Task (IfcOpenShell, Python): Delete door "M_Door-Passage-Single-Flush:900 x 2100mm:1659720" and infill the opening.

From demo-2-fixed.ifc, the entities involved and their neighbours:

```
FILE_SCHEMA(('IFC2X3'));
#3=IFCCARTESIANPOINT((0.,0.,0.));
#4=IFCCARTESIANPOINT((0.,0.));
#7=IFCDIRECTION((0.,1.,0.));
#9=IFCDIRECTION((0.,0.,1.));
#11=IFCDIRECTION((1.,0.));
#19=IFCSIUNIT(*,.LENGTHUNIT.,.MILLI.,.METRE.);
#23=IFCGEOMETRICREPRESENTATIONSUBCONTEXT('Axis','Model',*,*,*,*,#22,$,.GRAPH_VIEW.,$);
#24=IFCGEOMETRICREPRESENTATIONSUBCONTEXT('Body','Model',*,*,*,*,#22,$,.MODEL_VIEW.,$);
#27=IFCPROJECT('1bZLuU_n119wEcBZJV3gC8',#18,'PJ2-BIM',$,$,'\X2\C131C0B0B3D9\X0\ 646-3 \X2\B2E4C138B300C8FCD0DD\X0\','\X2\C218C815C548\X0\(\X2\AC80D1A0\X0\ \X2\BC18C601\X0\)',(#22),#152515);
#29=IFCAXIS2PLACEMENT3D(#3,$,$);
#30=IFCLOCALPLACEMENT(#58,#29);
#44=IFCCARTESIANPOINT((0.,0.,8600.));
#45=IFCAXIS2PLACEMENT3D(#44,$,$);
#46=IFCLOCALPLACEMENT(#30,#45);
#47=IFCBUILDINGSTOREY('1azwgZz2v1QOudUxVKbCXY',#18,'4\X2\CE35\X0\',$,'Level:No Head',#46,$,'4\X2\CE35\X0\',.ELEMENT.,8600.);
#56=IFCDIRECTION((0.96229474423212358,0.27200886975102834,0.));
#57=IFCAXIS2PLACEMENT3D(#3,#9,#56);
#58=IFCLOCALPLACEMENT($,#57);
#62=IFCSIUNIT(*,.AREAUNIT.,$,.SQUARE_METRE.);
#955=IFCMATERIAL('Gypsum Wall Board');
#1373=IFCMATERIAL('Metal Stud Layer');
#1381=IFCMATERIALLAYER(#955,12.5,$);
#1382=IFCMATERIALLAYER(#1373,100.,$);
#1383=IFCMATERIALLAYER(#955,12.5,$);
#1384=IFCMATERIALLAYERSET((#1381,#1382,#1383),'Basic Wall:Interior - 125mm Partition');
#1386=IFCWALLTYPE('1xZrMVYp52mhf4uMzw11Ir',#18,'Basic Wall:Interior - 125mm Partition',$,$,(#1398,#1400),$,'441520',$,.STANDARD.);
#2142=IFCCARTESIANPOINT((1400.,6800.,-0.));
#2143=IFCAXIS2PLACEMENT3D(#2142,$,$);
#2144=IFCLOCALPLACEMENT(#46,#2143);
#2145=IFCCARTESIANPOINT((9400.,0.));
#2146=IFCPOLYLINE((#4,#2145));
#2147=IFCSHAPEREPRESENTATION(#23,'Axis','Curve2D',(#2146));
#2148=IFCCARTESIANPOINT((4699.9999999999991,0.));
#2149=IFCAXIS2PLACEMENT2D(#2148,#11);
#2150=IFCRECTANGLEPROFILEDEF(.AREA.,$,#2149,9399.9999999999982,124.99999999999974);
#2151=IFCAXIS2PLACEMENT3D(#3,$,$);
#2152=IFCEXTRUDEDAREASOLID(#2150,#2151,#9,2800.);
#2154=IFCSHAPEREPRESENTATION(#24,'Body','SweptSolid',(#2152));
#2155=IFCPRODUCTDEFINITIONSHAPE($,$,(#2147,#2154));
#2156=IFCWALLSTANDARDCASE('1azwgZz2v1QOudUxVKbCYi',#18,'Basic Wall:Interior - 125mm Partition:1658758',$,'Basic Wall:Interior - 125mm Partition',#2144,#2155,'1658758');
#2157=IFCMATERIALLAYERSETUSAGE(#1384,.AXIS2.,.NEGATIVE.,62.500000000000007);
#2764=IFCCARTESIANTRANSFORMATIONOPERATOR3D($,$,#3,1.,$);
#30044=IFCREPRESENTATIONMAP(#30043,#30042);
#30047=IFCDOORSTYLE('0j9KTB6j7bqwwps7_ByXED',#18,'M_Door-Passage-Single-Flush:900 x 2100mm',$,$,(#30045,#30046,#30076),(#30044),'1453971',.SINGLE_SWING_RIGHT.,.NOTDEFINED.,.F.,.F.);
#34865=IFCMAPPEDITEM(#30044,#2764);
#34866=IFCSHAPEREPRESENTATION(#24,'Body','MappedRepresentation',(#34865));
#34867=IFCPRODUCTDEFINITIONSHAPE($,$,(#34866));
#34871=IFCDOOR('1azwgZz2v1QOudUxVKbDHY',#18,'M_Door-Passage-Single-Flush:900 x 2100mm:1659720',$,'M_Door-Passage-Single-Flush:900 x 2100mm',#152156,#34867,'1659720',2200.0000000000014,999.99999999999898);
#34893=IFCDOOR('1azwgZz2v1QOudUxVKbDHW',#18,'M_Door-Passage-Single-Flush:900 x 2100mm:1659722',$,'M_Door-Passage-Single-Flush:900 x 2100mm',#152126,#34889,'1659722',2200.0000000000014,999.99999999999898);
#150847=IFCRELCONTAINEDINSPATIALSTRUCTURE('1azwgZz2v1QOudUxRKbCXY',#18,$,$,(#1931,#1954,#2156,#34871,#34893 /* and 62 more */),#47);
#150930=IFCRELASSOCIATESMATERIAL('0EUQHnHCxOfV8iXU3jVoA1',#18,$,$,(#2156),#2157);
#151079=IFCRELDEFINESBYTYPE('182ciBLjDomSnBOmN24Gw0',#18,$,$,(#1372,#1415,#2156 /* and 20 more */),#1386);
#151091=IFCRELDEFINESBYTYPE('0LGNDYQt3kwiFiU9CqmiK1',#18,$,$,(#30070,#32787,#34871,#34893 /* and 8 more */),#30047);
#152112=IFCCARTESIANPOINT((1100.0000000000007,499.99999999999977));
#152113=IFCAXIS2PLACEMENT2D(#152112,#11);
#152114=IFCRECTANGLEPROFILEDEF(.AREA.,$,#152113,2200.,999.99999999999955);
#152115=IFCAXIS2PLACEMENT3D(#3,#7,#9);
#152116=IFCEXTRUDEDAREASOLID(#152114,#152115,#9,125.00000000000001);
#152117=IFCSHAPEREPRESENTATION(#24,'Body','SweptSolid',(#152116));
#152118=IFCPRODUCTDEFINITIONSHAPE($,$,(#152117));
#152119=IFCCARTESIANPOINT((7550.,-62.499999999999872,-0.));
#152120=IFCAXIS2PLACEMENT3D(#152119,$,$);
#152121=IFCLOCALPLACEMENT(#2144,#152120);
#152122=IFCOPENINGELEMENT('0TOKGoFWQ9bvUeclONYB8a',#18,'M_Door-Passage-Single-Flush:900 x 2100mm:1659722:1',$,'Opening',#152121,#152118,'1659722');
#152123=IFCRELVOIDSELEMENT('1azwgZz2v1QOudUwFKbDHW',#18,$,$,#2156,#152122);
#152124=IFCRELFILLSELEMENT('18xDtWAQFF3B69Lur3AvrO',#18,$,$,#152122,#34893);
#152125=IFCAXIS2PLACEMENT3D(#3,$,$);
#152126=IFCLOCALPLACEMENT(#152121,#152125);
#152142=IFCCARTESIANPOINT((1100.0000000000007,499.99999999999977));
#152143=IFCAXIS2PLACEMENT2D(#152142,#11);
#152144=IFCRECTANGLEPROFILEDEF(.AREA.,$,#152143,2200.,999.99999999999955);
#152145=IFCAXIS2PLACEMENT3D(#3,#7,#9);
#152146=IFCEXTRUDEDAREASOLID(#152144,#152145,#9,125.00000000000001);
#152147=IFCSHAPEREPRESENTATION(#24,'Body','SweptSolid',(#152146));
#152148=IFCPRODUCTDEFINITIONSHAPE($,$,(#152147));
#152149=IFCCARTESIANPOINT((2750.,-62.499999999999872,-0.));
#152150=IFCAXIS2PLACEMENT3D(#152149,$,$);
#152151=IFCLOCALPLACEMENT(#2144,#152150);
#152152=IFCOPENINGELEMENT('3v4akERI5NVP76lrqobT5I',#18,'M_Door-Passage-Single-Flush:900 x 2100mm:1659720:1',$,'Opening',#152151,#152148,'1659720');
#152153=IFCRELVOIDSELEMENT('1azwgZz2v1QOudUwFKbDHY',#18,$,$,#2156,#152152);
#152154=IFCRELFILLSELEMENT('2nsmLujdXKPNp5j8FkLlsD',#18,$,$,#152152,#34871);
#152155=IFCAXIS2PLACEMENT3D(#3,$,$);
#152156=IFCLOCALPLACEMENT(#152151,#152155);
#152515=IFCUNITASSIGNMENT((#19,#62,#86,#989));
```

```python
import ifcopenshell
import ifcopenshell.api.feature
import ifcopenshell.api.root
import ifcopenshell.geom
import ifcopenshell.util.shape

model = ifcopenshell.open("demo-2-fixed.ifc")
settings = ifcopenshell.geom.settings()


def volume(element):
    """Net volume in cubic metres, openings subtracted."""
    shape = ifcopenshell.geom.create_shape(settings, element)
    return ifcopenshell.util.shape.get_volume(shape.geometry)


door = model.by_id(34871)
opening = door.FillsVoids[0].RelatingOpeningElement
wall = opening.VoidsElements[0].RelatingBuildingElement
before = volume(wall)

ifcopenshell.api.root.remove_product(model, product=door)
ifcopenshell.api.feature.remove_feature(model, feature=opening)

after = volume(wall)

print(f"wall volume {before:.3f} -> {after:.3f} m3")

model.write("demo-2-fixed_v2.ifc")
```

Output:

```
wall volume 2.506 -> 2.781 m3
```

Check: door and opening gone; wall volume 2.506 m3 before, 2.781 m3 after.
